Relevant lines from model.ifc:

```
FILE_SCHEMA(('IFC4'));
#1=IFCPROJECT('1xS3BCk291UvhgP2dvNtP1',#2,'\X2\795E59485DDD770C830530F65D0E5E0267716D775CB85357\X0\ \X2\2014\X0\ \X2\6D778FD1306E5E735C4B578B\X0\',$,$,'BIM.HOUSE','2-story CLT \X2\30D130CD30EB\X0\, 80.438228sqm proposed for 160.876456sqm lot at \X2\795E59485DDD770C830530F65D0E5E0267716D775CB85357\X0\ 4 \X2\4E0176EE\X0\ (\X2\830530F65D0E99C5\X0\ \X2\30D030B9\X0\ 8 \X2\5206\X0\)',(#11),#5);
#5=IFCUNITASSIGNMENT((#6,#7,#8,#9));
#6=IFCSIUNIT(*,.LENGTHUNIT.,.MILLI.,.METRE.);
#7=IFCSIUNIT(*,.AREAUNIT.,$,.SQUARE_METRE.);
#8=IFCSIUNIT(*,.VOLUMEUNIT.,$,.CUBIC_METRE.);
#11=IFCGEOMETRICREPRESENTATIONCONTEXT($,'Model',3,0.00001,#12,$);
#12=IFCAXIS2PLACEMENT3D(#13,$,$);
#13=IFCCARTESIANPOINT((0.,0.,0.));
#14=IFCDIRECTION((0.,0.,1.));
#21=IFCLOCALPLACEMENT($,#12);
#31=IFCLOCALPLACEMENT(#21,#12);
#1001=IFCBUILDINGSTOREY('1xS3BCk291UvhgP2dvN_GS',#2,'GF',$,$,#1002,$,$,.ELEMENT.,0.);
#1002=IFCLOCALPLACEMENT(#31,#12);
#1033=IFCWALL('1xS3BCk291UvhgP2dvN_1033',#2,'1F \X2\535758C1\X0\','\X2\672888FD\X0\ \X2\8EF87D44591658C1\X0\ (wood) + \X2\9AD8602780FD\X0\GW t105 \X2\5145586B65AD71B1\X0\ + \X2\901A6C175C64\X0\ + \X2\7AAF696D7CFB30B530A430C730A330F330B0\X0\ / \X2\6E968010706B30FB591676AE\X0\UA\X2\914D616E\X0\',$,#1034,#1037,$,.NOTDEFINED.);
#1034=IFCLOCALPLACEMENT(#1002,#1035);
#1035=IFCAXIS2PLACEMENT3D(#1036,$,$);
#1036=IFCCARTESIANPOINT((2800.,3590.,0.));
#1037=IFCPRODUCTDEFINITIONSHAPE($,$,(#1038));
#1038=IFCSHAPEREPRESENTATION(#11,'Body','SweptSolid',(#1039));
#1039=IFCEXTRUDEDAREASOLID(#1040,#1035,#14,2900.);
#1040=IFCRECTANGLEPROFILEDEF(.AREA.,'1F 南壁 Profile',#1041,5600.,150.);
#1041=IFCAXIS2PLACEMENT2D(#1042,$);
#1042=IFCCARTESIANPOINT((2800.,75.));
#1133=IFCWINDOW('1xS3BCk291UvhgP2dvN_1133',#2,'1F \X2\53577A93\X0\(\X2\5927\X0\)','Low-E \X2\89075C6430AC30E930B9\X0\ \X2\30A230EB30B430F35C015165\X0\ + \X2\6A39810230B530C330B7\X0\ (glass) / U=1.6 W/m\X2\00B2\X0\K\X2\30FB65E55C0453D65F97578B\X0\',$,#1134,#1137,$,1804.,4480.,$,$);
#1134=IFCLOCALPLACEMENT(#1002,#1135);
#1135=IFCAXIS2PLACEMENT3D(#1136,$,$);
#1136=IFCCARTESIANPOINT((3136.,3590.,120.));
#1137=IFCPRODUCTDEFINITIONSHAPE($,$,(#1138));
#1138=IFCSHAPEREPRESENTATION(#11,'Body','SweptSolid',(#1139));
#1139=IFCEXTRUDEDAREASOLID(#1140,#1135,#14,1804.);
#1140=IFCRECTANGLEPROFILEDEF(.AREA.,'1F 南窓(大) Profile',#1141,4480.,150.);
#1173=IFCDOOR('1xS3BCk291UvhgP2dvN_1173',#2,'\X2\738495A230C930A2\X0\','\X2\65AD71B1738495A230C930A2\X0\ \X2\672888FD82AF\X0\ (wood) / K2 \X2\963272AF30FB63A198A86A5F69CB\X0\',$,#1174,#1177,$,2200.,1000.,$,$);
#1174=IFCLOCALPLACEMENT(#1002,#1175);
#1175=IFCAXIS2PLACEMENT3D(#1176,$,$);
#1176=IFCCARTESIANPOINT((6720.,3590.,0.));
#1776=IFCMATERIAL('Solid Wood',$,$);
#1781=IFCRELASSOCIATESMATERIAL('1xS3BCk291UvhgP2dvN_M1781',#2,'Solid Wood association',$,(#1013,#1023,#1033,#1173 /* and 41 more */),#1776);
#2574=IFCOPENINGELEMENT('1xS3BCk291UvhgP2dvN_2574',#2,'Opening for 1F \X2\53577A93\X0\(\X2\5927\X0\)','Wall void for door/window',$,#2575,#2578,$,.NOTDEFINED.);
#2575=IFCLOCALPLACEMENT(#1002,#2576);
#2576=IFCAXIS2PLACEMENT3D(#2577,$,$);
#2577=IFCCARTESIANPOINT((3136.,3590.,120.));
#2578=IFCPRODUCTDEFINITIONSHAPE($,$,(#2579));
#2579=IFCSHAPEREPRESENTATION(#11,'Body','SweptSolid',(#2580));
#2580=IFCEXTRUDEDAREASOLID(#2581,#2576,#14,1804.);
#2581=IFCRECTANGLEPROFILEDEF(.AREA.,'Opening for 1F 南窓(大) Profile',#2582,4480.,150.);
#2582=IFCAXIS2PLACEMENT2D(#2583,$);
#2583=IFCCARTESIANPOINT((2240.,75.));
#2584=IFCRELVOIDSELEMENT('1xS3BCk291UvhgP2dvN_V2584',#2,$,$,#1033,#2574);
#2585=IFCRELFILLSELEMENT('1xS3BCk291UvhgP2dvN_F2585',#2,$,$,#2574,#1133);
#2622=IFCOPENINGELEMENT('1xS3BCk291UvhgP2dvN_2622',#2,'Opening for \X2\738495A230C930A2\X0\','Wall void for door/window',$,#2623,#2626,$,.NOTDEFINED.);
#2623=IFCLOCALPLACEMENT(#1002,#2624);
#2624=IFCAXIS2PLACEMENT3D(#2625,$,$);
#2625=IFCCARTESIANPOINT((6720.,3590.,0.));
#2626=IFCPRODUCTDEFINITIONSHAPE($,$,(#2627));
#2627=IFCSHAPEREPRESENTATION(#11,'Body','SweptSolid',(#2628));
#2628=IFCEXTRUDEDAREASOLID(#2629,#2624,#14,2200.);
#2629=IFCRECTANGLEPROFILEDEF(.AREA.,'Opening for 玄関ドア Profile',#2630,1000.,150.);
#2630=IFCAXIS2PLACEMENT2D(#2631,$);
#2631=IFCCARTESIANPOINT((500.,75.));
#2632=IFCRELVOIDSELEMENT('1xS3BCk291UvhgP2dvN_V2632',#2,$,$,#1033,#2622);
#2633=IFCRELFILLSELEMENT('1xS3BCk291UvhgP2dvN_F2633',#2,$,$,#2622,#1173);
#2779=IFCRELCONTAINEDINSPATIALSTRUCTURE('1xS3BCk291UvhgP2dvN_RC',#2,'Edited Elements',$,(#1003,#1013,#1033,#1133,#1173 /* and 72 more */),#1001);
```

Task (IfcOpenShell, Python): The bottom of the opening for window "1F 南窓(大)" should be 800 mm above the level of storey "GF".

```python
import numpy as np
import ifcopenshell
import ifcopenshell.api.geometry
import ifcopenshell.geom
import ifcopenshell.util.element
import ifcopenshell.util.placement
import ifcopenshell.util.shape
import ifcopenshell.util.unit

model = ifcopenshell.open("model.ifc")
unit_scale = ifcopenshell.util.unit.calculate_unit_scale(model)

window = model.by_id(1133)
opening = window.FillsVoids[0].RelatingOpeningElement
storey = ifcopenshell.util.element.get_container(window, ifc_class="IfcBuildingStorey")
level = ifcopenshell.util.placement.get_local_placement(storey.ObjectPlacement)[2, 3]

# The opening's origin need not be at the sill, so measure its lowest point.
shape = ifcopenshell.geom.create_shape(ifcopenshell.geom.settings(), opening)
bottom = ifcopenshell.util.shape.get_shape_bottom_elevation(shape, shape.geometry) / unit_scale
dz = level + 800.0 - bottom

shift = np.array([0.0, 0.0, dz])
# The window is not placed relative to its opening, so move both.
for product in (opening, window):
    matrix = ifcopenshell.util.placement.get_local_placement(product.ObjectPlacement)
    matrix[:3, 3] += shift
    ifcopenshell.api.geometry.edit_object_placement(model, product=product, matrix=matrix, is_si=False)

print(f"moved by {dz * unit_scale:+.3f} m")

model.write("model_edited.ifc")
```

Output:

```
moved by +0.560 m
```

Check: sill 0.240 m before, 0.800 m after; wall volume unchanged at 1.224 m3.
